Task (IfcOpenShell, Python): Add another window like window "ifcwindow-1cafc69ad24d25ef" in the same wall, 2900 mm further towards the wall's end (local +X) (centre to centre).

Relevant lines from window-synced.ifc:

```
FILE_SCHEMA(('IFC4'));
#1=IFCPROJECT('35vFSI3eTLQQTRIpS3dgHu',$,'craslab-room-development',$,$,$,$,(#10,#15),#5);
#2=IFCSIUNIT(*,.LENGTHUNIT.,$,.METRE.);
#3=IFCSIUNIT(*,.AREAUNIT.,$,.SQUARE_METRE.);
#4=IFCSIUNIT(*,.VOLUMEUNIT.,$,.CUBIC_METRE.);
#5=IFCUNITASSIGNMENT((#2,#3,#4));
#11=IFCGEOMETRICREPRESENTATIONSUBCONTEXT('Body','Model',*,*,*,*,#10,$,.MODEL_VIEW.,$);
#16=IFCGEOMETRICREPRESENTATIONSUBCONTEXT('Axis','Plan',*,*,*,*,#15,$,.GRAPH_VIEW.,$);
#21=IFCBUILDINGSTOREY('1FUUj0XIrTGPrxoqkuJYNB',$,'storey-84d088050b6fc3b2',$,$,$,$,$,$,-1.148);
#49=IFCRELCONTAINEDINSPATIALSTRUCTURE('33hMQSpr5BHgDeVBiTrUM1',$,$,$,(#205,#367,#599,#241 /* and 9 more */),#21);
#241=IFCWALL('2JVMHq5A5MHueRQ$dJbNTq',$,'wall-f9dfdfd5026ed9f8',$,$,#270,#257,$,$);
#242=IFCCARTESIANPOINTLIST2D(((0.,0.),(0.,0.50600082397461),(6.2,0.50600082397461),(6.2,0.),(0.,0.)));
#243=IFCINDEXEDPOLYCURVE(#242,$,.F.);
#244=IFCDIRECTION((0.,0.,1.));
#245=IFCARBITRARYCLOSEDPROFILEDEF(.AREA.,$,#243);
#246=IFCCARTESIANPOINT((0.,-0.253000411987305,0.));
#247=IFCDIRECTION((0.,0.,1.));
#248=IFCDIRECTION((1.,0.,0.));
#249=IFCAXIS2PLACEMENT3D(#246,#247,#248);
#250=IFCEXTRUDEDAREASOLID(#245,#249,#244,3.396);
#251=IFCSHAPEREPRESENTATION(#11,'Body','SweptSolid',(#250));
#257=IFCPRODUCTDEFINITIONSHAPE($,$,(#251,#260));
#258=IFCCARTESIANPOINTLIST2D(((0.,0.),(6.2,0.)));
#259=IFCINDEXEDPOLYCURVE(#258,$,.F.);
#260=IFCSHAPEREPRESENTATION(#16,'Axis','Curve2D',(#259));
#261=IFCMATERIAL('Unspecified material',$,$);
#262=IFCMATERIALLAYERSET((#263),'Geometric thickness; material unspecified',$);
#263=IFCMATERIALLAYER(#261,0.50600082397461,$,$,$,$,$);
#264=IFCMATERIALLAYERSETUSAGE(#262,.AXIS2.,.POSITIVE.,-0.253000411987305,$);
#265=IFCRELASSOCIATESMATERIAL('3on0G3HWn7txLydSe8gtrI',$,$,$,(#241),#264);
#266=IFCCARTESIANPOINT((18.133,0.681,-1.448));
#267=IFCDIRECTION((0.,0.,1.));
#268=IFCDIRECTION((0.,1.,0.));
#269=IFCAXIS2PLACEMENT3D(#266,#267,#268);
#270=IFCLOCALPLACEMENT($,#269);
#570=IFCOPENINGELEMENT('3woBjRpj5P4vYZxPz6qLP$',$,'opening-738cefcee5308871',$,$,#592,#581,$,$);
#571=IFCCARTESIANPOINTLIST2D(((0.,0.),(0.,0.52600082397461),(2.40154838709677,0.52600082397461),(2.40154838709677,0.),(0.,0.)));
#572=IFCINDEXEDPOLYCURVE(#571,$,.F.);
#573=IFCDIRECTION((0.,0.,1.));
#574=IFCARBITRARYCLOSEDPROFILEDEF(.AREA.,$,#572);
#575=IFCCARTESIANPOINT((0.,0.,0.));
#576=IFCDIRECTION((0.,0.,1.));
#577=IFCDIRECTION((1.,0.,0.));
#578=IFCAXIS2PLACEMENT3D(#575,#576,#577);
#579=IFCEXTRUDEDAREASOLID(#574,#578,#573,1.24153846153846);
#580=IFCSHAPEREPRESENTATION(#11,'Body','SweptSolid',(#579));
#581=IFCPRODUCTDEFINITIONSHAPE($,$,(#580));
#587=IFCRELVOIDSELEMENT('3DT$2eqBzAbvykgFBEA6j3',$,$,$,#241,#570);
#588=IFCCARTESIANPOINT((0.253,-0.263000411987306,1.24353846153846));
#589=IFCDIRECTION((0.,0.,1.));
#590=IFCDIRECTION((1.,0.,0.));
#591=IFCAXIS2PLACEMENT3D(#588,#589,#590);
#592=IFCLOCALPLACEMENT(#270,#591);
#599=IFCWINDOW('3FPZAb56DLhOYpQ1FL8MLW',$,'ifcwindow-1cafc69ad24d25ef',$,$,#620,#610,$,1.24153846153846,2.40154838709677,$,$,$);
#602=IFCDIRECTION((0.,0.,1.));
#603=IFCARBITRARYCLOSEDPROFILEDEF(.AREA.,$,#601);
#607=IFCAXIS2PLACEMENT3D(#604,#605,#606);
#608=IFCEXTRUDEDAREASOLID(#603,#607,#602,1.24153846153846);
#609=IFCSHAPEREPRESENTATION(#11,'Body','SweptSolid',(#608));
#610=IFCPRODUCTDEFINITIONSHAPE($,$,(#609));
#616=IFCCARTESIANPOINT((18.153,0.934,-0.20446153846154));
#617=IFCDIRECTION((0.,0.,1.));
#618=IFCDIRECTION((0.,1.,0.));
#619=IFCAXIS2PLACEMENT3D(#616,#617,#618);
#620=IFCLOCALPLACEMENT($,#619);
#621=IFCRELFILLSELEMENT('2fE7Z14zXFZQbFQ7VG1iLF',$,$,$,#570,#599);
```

```python
import ifcopenshell
import ifcopenshell.api.feature
import ifcopenshell.api.geometry
import ifcopenshell.api.root
import ifcopenshell.geom
import ifcopenshell.util.element
import ifcopenshell.util.placement
import ifcopenshell.util.shape
import ifcopenshell.util.unit

model = ifcopenshell.open("window-synced.ifc")
unit_scale = ifcopenshell.util.unit.calculate_unit_scale(model)
settings = ifcopenshell.geom.settings()


def volume(element):
    """Net volume in cubic metres, openings subtracted."""
    shape = ifcopenshell.geom.create_shape(settings, element)
    return ifcopenshell.util.shape.get_volume(shape.geometry)


window = model.by_guid("3FPZAb56DLhOYpQ1FL8MLW")
opening = window.FillsVoids[0].RelatingOpeningElement
wall = opening.VoidsElements[0].RelatingBuildingElement
before = volume(wall)
shift = ifcopenshell.util.placement.get_local_placement(wall.ObjectPlacement)[:3, 0] * 2.9 / unit_scale

# copy_class copies the void relationship, type, container and properties, but no geometry.
new_opening = ifcopenshell.api.root.copy_class(model, product=opening)
new_opening.Representation = ifcopenshell.util.element.copy_deep(
    model, opening.Representation, exclude=["IfcGeometricRepresentationContext", "IfcRepresentationMap"]
)
new_window = ifcopenshell.api.root.copy_class(model, product=window)
new_window.Representation = ifcopenshell.util.element.copy_deep(
    model, window.Representation, exclude=["IfcGeometricRepresentationContext", "IfcRepresentationMap"]
)
ifcopenshell.api.feature.add_filling(model, opening=new_opening, element=new_window)

for old, new in ((opening, new_opening), (window, new_window)):
    matrix = ifcopenshell.util.placement.get_local_placement(old.ObjectPlacement)
    matrix[:3, 3] += shift
    ifcopenshell.api.geometry.edit_object_placement(model, product=new, matrix=matrix, is_si=False)

after = volume(wall)

print(f"wall volume {before:.3f} -> {after:.3f} m3")

model.write("window-synced_rev.ifc")
```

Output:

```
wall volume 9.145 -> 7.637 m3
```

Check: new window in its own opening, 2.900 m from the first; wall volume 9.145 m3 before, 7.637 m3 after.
